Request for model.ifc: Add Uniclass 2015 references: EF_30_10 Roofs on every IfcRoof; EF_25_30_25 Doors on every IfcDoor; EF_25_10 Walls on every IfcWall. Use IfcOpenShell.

First a look at what the model holds.

```python
import ifcopenshell

model = ifcopenshell.open("model.ifc")
print(model.schema)
print("classifications:", [c.Name for c in model.by_type("IfcClassification")])
for ifc_class in ("IfcDoor", "IfcRoof", "IfcStair", "IfcWall", "IfcWindow"):
    print(ifc_class, len(model.by_type(ifc_class)))
```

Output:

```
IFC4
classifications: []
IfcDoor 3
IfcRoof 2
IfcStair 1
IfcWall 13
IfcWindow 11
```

```python
import ifcopenshell
import ifcopenshell.api.classification

model = ifcopenshell.open("model.ifc")

system = ifcopenshell.api.classification.add_classification(model, classification="Uniclass 2015")

codes = {
    "IfcRoof": ("EF_30_10", "Roofs"),
    "IfcDoor": ("EF_25_30_25", "Doors"),
    "IfcWall": ("EF_25_10", "Walls"),
}
for ifc_class, (code, name) in codes.items():
    products = model.by_type(ifc_class)
    ifcopenshell.api.classification.add_reference(
        model, products=products, classification=system, identification=code, name=name
    )
    print(code, len(products))

model.write("model_rev.ifc")
```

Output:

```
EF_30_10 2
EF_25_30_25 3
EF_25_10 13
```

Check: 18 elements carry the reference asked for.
